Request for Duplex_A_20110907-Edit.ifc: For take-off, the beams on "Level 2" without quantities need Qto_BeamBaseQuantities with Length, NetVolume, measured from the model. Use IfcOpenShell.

First a look at what the model holds.

```python
import ifcopenshell
import ifcopenshell.util.element
import ifcopenshell.util.unit

model = ifcopenshell.open("Duplex_A_20110907-Edit.ifc")
print(model.schema)
for unit_type in ("LENGTHUNIT", "AREAUNIT", "VOLUMEUNIT"):
    print(unit_type, ifcopenshell.util.unit.calculate_unit_scale(model, unit_type))
storey = next(s for s in model.by_type("IfcBuildingStorey") if s.Name == "Level 2")
beams = [e for e in ifcopenshell.util.element.get_decomposition(storey) if e.is_a("IfcBeam")]
for e in sorted(beams, key=lambda e: e.id()):
    print(e.id(), e.is_a(), e.Name, list(ifcopenshell.util.element.get_psets(e, qtos_only=True)), sep=" | ")
```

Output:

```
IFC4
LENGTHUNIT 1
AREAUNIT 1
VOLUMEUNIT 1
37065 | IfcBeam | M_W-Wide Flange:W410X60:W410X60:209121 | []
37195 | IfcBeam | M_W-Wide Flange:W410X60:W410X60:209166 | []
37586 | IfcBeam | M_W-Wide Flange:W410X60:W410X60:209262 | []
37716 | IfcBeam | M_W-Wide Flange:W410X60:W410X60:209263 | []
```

```python
import ifcopenshell
import ifcopenshell.api.pset
import ifcopenshell.geom
import ifcopenshell.util.element
import ifcopenshell.util.shape
import ifcopenshell.util.unit

model = ifcopenshell.open("Duplex_A_20110907-Edit.ifc")
unit_scale = ifcopenshell.util.unit.calculate_unit_scale(model)
volume_scale = ifcopenshell.util.unit.calculate_unit_scale(model, "VOLUMEUNIT")
settings = ifcopenshell.geom.settings()

storey = next(s for s in model.by_type("IfcBuildingStorey") if s.Name == "Level 2")
beams = [e for e in ifcopenshell.util.element.get_decomposition(storey) if e.is_a("IfcBeam")]

for e in sorted(beams, key=lambda e: e.id()):
    if ifcopenshell.util.element.get_psets(e, qtos_only=True, should_inherit=False):
        continue
    # Geometry comes back in metres, in the element's own axes.
    shape = ifcopenshell.geom.create_shape(settings, e)
    values = {
        "Length": ifcopenshell.util.shape.get_max_xyz(shape.geometry) / unit_scale,
        "NetVolume": ifcopenshell.util.shape.get_volume(shape.geometry) / volume_scale,
    }
    qto = ifcopenshell.api.pset.add_qto(model, product=e, name="Qto_BeamBaseQuantities")
    ifcopenshell.api.pset.edit_qto(model, qto=qto, properties=values)
    print(e.id(), {k: round(v, 3) for k, v in values.items()})

model.write("Duplex_A_20110907-Edit_v2.ifc")
```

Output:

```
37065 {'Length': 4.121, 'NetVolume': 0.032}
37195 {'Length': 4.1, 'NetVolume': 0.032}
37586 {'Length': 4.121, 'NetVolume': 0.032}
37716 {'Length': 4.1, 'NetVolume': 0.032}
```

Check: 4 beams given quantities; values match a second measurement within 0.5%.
